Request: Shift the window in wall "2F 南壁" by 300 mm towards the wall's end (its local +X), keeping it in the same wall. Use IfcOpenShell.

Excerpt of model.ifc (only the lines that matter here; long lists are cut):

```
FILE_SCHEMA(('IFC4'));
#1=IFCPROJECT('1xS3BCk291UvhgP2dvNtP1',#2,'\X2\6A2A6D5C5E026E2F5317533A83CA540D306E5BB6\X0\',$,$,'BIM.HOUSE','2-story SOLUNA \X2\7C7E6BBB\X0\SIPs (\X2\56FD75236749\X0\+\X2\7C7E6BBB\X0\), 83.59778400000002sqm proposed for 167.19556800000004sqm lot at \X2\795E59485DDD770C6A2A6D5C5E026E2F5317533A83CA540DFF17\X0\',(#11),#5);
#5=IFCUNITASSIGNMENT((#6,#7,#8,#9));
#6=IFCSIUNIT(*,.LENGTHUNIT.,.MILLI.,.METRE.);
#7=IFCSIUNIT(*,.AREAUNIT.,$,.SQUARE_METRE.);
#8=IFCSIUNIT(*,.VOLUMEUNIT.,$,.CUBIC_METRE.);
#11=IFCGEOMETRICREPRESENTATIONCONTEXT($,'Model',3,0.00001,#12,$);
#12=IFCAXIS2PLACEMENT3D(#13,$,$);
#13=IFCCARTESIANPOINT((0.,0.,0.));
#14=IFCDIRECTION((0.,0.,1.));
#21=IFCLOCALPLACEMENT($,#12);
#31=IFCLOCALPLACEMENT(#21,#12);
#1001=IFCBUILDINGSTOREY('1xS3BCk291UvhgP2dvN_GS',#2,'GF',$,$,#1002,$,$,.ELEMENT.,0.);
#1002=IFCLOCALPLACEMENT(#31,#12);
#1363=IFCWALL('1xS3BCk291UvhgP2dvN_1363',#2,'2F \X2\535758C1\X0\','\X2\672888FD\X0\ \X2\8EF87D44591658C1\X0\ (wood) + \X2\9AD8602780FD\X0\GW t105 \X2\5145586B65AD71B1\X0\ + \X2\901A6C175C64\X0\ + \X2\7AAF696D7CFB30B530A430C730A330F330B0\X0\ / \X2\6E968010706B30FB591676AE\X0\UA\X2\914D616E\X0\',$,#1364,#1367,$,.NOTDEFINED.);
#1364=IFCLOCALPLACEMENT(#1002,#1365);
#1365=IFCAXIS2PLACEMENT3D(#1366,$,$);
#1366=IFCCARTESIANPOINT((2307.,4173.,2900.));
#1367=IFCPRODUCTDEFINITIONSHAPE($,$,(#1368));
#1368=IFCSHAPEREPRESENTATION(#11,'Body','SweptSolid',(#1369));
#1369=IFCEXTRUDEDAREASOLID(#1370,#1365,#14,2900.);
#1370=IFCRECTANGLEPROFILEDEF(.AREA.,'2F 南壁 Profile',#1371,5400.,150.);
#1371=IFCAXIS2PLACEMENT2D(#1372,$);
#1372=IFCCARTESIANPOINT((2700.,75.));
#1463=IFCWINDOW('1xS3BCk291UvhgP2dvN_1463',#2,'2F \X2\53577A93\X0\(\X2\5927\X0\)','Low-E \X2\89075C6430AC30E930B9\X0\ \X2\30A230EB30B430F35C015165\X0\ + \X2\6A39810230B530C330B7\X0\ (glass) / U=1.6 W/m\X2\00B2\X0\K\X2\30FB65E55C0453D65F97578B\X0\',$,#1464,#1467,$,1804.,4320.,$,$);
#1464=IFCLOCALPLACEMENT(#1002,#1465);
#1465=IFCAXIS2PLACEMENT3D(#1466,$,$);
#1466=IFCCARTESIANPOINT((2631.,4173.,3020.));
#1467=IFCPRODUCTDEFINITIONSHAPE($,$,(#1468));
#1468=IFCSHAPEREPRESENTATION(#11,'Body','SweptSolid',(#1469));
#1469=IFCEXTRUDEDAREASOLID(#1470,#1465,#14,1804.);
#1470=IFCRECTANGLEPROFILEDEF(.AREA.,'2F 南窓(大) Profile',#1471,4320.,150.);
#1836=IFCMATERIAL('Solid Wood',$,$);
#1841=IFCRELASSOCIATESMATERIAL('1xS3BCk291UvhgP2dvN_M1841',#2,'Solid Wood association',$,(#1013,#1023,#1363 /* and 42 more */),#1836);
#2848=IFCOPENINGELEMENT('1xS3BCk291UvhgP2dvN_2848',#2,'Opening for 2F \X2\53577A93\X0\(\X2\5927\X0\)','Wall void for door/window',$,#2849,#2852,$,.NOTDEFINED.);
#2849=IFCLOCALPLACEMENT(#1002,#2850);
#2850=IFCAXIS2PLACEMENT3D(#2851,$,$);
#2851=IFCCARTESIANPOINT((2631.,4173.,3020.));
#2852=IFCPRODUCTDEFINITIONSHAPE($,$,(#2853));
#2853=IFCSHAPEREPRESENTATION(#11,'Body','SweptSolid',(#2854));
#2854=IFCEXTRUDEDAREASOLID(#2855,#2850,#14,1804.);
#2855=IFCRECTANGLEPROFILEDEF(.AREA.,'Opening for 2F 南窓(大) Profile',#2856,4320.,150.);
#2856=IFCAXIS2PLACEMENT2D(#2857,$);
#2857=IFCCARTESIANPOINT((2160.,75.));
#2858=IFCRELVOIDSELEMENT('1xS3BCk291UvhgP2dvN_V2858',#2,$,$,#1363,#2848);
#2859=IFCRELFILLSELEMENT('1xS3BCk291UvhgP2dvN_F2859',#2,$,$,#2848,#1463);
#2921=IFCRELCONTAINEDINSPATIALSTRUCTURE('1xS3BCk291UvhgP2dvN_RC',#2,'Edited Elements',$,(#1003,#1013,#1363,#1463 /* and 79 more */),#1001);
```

```python
import ifcopenshell
import ifcopenshell.api.geometry
import ifcopenshell.util.placement
import ifcopenshell.util.unit

model = ifcopenshell.open("model.ifc")
unit_scale = ifcopenshell.util.unit.calculate_unit_scale(model)

window = model.by_id(1463)
opening = window.FillsVoids[0].RelatingOpeningElement
wall = opening.VoidsElements[0].RelatingBuildingElement

wall_matrix = ifcopenshell.util.placement.get_local_placement(wall.ObjectPlacement)
shift = wall_matrix[:3, 0] * 0.3 / unit_scale
before = ifcopenshell.util.placement.get_local_placement(window.ObjectPlacement)[:3, 3].copy()

# The window is not placed relative to its opening, so move both.
for product in (opening, window):
    matrix = ifcopenshell.util.placement.get_local_placement(product.ObjectPlacement)
    matrix[:3, 3] += shift
    ifcopenshell.api.geometry.edit_object_placement(model, product=product, matrix=matrix, is_si=False)

after = ifcopenshell.util.placement.get_local_placement(window.ObjectPlacement)[:3, 3]
print("window moved by", (after - before).round(3) + 0.0)

model.write("model_rev.ifc")
```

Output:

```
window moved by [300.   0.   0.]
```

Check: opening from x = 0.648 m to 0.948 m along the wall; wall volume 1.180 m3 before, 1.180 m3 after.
